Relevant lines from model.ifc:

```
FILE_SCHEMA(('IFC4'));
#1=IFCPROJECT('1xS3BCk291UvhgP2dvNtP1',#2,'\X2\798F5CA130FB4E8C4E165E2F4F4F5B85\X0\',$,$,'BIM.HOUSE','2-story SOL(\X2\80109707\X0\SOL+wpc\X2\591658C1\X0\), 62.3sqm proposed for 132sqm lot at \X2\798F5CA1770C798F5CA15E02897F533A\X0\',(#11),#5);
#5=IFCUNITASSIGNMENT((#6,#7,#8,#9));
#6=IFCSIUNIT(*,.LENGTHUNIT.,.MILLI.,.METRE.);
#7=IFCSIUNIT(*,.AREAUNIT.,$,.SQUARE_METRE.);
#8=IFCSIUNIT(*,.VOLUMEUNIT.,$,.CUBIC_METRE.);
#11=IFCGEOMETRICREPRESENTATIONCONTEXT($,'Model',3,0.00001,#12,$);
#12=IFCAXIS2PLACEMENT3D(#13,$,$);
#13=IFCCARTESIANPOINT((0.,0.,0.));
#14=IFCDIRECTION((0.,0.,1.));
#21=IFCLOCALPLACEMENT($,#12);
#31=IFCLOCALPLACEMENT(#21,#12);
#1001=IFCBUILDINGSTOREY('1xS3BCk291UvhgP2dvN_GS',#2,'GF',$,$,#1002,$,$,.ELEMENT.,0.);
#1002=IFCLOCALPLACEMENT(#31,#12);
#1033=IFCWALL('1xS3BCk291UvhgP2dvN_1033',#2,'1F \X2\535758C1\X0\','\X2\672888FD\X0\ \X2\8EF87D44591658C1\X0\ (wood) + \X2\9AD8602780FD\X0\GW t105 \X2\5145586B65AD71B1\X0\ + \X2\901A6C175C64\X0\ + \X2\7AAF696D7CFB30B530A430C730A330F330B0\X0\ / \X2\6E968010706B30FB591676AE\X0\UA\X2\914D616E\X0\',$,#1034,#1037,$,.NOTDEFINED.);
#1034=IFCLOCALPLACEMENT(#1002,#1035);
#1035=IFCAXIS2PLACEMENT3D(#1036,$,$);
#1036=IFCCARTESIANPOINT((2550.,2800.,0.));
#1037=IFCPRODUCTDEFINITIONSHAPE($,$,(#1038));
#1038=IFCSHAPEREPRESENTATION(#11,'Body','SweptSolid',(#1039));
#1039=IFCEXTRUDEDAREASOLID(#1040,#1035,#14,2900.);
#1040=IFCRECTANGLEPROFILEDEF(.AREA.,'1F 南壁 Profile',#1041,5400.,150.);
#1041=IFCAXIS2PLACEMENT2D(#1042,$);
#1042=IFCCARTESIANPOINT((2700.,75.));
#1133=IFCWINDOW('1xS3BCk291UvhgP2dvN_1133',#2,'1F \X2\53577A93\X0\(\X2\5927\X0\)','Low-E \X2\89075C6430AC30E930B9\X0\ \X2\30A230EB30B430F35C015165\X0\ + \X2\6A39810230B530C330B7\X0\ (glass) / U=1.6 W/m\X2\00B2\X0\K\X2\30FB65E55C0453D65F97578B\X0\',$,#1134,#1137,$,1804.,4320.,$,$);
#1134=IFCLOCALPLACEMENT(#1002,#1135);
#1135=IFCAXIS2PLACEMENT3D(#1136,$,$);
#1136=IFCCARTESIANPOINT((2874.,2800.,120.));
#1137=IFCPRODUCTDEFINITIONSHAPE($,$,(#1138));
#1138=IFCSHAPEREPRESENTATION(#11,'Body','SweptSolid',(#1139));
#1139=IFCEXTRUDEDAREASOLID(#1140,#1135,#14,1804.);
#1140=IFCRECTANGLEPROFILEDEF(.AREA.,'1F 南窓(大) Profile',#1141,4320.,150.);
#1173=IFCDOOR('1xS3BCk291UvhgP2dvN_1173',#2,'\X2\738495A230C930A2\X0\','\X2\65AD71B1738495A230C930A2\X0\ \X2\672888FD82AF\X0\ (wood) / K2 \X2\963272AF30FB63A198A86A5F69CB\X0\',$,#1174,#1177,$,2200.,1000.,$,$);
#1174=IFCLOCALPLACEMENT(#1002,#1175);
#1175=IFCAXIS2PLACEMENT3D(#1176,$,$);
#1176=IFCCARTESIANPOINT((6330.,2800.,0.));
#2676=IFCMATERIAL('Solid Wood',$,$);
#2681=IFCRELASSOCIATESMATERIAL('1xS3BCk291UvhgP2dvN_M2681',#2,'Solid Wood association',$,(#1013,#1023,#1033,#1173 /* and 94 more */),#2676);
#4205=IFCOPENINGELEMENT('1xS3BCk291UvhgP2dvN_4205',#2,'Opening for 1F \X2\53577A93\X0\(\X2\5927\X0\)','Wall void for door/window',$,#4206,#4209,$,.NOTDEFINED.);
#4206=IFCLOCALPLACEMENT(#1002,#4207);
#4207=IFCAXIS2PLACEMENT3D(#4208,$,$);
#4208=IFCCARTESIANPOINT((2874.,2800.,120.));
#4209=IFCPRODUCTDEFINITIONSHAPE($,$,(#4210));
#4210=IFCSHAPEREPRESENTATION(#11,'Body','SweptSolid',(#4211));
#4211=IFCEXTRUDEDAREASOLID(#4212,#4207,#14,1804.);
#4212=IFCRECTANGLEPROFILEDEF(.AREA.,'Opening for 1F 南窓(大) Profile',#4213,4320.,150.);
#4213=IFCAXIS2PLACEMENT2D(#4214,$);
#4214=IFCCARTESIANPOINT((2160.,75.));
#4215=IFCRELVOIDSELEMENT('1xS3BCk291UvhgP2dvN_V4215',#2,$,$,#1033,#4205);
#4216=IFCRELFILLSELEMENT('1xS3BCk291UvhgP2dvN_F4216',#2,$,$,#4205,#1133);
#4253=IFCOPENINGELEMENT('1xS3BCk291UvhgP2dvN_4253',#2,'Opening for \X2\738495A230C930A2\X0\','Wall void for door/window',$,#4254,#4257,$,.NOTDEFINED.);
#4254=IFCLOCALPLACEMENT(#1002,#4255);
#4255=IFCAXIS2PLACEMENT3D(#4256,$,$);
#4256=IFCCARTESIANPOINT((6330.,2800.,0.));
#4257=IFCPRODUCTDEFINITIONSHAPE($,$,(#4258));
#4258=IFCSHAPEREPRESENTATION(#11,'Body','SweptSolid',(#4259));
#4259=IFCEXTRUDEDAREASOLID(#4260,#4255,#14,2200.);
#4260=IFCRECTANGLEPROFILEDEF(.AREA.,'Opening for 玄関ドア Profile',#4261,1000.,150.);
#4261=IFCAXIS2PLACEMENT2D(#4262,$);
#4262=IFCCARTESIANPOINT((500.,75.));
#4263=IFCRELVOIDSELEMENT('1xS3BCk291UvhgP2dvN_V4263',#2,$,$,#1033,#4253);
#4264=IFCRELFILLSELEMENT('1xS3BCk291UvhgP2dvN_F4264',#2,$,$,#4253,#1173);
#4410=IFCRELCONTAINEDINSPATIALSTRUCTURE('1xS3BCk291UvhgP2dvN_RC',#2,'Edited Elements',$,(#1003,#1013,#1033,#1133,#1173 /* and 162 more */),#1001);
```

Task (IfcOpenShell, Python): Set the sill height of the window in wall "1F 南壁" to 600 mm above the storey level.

```python
import numpy as np
import ifcopenshell
import ifcopenshell.api.geometry
import ifcopenshell.geom
import ifcopenshell.util.element
import ifcopenshell.util.placement
import ifcopenshell.util.shape
import ifcopenshell.util.unit

model = ifcopenshell.open("model.ifc")
unit_scale = ifcopenshell.util.unit.calculate_unit_scale(model)

window = model.by_guid("1xS3BCk291UvhgP2dvN_1133")
opening = window.FillsVoids[0].RelatingOpeningElement
storey = ifcopenshell.util.element.get_container(window, ifc_class="IfcBuildingStorey")
level = ifcopenshell.util.placement.get_local_placement(storey.ObjectPlacement)[2, 3]

# The opening's origin need not be at the sill, so measure its lowest point.
shape = ifcopenshell.geom.create_shape(ifcopenshell.geom.settings(), opening)
bottom = ifcopenshell.util.shape.get_shape_bottom_elevation(shape, shape.geometry) / unit_scale
dz = level + 0.6 / unit_scale - bottom

shift = np.array([0.0, 0.0, dz])
# The window is not placed relative to its opening, so move both.
for product in (opening, window):
    matrix = ifcopenshell.util.placement.get_local_placement(product.ObjectPlacement)
    matrix[:3, 3] += shift
    ifcopenshell.api.geometry.edit_object_placement(model, product=product, matrix=matrix, is_si=False)

print(f"moved by {dz * unit_scale:+.3f} m")

model.write("model_edited.ifc")
```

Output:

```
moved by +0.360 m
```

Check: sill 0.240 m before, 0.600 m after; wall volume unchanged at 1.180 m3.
